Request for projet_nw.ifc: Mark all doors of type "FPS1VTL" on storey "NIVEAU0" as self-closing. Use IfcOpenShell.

First a look at what the model holds.

```python
import ifcopenshell
import ifcopenshell.util.element

model = ifcopenshell.open("projet_nw.ifc")
print(model.schema)
storey = next(s for s in model.by_type("IfcBuildingStorey") if s.Name == "NIVEAU0")
doors = [e for e in ifcopenshell.util.element.get_decomposition(storey) if e.is_a("IfcDoor")]
seen = {}
for e in doors:
    element_type = ifcopenshell.util.element.get_type(e)
    key = (element_type.Name if element_type != e and element_type else None, ifcopenshell.util.element.get_pset(e, "Pset_DoorCommon", "SelfClosing"))
    seen[key] = seen.get(key, 0) + 1
for (name, value), count in sorted(seen.items(), key=str):
    print(count, "x", name, "|", value)
```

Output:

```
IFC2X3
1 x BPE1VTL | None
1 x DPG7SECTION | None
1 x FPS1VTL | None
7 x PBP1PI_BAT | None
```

```python
import ifcopenshell
import ifcopenshell.api.pset
import ifcopenshell.util.element

model = ifcopenshell.open("projet_nw.ifc")

storey = next(s for s in model.by_type("IfcBuildingStorey") if s.Name == "NIVEAU0")
doors = [e for e in ifcopenshell.util.element.get_decomposition(storey) if e.is_a("IfcDoor")]

count = 0
for e in doors:
    element_type = ifcopenshell.util.element.get_type(e)
    if element_type in (None, e) or element_type.Name != "FPS1VTL":
        continue
    # add_pset returns the element's existing set when there is one.
    pset = ifcopenshell.api.pset.add_pset(model, product=e, name="Pset_DoorCommon")
    ifcopenshell.api.pset.edit_pset(model, pset=pset, properties={"SelfClosing": True})
    count += 1

print(count, "doors updated")

model.write("projet_nw_edited.ifc")
```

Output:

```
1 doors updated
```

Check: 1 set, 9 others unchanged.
